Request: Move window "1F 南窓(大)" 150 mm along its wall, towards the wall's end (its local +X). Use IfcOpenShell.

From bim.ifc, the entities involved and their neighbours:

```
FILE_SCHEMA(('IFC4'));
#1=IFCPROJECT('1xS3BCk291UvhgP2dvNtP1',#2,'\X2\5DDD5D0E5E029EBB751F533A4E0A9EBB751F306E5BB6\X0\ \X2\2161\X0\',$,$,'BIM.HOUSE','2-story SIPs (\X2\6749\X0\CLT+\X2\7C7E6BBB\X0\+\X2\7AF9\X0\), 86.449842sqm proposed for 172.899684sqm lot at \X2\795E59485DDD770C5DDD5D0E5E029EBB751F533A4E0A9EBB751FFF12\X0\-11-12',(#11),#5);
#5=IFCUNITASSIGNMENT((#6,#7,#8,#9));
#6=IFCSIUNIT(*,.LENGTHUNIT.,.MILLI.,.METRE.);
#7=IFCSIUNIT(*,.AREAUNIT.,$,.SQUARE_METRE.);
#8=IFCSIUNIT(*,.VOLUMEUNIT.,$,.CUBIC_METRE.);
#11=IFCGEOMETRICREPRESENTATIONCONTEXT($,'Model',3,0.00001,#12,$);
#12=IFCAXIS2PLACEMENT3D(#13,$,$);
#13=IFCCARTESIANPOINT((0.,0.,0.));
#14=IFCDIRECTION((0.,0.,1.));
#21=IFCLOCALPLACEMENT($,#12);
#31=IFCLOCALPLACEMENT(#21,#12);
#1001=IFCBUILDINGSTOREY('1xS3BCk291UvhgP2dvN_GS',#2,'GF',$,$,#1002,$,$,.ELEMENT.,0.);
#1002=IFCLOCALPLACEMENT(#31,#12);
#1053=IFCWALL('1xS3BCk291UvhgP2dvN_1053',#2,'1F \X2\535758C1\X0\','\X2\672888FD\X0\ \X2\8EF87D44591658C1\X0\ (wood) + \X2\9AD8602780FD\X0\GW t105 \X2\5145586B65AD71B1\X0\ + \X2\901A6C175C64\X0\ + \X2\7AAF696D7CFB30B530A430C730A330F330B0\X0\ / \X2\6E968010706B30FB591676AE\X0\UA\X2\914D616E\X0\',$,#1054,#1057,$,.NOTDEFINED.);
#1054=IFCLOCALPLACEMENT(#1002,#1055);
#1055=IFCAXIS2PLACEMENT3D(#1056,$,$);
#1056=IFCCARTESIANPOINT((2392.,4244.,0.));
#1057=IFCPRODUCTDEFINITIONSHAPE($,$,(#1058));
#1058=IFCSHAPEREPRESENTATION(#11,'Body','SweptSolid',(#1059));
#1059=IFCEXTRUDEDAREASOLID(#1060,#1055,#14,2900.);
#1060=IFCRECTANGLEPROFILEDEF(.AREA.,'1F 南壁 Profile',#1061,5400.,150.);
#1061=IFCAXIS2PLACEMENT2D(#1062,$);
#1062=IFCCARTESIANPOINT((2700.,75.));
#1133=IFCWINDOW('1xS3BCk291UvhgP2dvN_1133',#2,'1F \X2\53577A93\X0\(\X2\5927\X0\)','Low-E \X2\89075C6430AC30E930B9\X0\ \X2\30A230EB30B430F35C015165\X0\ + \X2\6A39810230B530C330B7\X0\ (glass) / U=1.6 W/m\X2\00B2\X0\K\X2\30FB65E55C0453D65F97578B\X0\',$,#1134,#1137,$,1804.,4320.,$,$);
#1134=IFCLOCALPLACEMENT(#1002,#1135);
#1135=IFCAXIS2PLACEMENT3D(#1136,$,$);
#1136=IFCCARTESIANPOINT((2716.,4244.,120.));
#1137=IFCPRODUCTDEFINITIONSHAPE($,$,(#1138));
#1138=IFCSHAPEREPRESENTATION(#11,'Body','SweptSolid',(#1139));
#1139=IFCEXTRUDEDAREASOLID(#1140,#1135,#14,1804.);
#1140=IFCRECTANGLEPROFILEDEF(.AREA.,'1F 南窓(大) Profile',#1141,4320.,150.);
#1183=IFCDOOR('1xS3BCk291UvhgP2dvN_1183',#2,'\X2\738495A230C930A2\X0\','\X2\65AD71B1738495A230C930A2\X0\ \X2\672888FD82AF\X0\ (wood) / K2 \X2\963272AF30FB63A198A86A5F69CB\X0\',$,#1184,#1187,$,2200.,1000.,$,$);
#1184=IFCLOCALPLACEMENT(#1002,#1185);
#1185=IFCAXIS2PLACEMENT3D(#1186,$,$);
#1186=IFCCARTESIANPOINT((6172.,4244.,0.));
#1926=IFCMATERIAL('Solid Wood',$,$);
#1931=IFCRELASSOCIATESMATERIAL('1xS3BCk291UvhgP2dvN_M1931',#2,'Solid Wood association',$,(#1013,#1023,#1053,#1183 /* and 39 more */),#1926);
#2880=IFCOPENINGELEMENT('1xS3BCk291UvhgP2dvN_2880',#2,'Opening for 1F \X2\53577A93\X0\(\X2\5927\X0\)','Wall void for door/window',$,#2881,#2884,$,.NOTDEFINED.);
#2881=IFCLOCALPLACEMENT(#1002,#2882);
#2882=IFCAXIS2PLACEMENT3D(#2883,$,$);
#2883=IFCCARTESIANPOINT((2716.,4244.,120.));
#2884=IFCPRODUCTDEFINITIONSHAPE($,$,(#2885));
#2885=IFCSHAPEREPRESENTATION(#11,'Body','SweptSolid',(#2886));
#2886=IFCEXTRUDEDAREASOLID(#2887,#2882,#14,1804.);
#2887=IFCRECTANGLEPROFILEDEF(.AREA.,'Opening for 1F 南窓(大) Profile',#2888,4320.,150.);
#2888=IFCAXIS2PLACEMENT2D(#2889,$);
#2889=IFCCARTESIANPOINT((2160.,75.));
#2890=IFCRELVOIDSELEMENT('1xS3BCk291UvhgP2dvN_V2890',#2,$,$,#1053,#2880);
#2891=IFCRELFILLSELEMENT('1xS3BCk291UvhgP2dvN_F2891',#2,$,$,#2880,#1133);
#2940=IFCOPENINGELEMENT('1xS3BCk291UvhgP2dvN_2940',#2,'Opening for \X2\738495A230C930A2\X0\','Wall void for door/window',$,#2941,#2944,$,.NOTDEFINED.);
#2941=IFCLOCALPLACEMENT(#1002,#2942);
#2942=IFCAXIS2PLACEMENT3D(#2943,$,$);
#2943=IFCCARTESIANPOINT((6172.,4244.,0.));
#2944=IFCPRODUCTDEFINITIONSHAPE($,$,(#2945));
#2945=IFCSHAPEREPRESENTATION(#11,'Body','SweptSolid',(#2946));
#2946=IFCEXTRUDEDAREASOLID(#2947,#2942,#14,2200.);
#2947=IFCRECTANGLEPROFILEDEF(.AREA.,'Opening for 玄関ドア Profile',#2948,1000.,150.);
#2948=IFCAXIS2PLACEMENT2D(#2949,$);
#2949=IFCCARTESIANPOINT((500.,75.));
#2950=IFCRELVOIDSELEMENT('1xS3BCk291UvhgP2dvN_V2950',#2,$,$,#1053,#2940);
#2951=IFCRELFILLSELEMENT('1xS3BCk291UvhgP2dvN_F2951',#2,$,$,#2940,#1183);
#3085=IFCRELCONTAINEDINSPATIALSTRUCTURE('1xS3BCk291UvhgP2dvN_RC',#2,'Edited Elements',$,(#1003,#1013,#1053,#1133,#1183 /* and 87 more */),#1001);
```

```python
import ifcopenshell
import ifcopenshell.api.geometry
import ifcopenshell.util.placement
import ifcopenshell.util.unit

model = ifcopenshell.open("bim.ifc")
unit_scale = ifcopenshell.util.unit.calculate_unit_scale(model)

window = model.by_id(1133)
opening = window.FillsVoids[0].RelatingOpeningElement
wall = opening.VoidsElements[0].RelatingBuildingElement

wall_matrix = ifcopenshell.util.placement.get_local_placement(wall.ObjectPlacement)
shift = wall_matrix[:3, 0] * 0.15 / unit_scale
before = ifcopenshell.util.placement.get_local_placement(window.ObjectPlacement)[:3, 3].copy()

# The window is not placed relative to its opening, so move both.
for product in (opening, window):
    matrix = ifcopenshell.util.placement.get_local_placement(product.ObjectPlacement)
    matrix[:3, 3] += shift
    ifcopenshell.api.geometry.edit_object_placement(model, product=product, matrix=matrix, is_si=False)

after = ifcopenshell.util.placement.get_local_placement(window.ObjectPlacement)[:3, 3]
print("window moved by", (after - before).round(3) + 0.0)

model.write("bim_updated.ifc")
```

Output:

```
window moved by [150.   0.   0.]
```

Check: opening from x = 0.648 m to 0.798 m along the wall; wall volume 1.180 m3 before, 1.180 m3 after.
